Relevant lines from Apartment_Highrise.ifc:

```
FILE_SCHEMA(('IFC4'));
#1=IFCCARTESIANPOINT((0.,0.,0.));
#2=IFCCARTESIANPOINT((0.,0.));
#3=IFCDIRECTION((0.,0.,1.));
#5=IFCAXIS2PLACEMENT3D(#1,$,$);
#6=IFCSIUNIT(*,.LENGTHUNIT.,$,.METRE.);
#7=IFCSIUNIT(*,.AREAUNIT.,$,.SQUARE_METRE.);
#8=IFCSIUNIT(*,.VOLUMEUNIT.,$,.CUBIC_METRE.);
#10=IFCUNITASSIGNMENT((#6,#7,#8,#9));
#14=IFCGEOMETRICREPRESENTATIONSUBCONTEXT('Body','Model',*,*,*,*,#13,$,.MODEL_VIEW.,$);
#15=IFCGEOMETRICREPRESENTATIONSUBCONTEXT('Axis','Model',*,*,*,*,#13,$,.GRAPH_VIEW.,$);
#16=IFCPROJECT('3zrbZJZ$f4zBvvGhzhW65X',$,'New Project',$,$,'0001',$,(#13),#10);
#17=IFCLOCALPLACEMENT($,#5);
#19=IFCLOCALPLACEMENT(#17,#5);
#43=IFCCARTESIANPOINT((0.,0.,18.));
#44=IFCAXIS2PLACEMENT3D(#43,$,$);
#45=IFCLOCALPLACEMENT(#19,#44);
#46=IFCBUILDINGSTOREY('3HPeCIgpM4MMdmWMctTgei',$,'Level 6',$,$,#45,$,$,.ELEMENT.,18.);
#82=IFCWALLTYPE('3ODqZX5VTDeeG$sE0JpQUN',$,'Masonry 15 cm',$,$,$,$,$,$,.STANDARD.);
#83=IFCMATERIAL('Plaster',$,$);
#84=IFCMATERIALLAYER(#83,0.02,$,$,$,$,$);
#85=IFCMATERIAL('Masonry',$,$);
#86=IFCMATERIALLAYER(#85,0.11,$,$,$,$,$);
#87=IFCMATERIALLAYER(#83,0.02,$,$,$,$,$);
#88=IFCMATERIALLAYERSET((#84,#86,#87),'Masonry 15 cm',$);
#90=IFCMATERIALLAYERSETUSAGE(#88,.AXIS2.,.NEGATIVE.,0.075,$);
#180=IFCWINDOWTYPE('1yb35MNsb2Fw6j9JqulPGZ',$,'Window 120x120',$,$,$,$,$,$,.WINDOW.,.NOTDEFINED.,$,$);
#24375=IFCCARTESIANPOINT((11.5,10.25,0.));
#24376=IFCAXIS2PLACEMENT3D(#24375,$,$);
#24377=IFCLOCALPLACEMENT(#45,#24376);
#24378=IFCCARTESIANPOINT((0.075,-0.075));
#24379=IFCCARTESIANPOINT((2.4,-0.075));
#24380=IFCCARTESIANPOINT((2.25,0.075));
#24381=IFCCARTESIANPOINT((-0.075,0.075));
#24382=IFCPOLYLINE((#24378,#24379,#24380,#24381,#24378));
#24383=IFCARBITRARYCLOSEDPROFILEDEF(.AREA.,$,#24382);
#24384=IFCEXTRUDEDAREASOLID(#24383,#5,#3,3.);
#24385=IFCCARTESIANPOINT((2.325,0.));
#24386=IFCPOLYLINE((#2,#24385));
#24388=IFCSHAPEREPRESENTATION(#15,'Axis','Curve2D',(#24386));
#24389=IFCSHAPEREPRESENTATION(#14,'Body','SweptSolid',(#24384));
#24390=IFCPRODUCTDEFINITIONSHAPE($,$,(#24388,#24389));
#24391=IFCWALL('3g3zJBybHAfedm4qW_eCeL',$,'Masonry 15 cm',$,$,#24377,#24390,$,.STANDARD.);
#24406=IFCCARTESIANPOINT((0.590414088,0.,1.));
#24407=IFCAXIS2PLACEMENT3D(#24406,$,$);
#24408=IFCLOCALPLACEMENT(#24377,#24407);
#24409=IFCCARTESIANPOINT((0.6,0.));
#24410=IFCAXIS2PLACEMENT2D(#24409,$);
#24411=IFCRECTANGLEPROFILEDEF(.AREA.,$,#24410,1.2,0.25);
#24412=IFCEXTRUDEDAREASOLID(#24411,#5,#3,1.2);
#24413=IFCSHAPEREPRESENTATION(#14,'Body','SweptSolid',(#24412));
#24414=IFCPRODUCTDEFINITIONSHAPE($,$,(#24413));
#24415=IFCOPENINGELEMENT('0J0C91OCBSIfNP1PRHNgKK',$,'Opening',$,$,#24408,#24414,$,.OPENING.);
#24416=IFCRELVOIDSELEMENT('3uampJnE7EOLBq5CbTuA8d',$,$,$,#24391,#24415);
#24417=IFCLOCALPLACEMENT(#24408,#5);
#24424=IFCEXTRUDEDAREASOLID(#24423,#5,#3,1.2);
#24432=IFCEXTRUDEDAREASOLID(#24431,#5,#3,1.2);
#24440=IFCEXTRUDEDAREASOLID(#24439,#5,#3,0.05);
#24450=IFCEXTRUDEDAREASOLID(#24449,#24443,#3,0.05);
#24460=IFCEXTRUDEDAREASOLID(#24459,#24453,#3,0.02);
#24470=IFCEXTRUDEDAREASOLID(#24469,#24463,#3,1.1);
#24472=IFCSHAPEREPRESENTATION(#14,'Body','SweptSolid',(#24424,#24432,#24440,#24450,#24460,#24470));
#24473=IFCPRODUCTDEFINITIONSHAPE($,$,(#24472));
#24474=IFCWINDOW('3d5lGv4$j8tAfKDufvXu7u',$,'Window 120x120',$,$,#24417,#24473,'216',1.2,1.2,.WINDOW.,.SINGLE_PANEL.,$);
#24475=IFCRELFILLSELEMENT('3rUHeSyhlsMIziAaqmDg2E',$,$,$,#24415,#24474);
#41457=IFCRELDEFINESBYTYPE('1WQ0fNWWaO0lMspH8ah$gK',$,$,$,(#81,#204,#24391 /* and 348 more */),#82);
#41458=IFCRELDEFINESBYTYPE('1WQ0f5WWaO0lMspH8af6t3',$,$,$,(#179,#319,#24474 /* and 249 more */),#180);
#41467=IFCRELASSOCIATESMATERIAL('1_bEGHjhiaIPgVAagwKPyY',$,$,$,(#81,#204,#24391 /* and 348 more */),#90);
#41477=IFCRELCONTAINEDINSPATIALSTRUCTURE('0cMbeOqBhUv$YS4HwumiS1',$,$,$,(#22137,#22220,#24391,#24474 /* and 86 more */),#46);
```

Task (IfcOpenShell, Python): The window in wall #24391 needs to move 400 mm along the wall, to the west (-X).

```python
import ifcopenshell
import ifcopenshell.api.geometry
import ifcopenshell.util.placement
import ifcopenshell.util.unit

model = ifcopenshell.open("Apartment_Highrise.ifc")
unit_scale = ifcopenshell.util.unit.calculate_unit_scale(model)

window = model.by_guid("3d5lGv4$j8tAfKDufvXu7u")
opening = window.FillsVoids[0].RelatingOpeningElement
wall = opening.VoidsElements[0].RelatingBuildingElement

wall_matrix = ifcopenshell.util.placement.get_local_placement(wall.ObjectPlacement)
shift = wall_matrix[:3, 0] * -0.4 / unit_scale
before = ifcopenshell.util.placement.get_local_placement(window.ObjectPlacement)[:3, 3].copy()

# The window is placed relative to its opening, so it follows when the opening moves.
matrix = ifcopenshell.util.placement.get_local_placement(opening.ObjectPlacement)
matrix[:3, 3] += shift
ifcopenshell.api.geometry.edit_object_placement(
    model, product=opening, matrix=matrix, is_si=False, should_transform_children=True
)

after = ifcopenshell.util.placement.get_local_placement(window.ObjectPlacement)[:3, 3]
print("window moved by", (after - before).round(3) + 0.0)

model.write("Apartment_Highrise_edited.ifc")
```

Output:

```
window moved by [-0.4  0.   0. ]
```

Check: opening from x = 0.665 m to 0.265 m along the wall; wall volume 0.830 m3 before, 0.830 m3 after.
